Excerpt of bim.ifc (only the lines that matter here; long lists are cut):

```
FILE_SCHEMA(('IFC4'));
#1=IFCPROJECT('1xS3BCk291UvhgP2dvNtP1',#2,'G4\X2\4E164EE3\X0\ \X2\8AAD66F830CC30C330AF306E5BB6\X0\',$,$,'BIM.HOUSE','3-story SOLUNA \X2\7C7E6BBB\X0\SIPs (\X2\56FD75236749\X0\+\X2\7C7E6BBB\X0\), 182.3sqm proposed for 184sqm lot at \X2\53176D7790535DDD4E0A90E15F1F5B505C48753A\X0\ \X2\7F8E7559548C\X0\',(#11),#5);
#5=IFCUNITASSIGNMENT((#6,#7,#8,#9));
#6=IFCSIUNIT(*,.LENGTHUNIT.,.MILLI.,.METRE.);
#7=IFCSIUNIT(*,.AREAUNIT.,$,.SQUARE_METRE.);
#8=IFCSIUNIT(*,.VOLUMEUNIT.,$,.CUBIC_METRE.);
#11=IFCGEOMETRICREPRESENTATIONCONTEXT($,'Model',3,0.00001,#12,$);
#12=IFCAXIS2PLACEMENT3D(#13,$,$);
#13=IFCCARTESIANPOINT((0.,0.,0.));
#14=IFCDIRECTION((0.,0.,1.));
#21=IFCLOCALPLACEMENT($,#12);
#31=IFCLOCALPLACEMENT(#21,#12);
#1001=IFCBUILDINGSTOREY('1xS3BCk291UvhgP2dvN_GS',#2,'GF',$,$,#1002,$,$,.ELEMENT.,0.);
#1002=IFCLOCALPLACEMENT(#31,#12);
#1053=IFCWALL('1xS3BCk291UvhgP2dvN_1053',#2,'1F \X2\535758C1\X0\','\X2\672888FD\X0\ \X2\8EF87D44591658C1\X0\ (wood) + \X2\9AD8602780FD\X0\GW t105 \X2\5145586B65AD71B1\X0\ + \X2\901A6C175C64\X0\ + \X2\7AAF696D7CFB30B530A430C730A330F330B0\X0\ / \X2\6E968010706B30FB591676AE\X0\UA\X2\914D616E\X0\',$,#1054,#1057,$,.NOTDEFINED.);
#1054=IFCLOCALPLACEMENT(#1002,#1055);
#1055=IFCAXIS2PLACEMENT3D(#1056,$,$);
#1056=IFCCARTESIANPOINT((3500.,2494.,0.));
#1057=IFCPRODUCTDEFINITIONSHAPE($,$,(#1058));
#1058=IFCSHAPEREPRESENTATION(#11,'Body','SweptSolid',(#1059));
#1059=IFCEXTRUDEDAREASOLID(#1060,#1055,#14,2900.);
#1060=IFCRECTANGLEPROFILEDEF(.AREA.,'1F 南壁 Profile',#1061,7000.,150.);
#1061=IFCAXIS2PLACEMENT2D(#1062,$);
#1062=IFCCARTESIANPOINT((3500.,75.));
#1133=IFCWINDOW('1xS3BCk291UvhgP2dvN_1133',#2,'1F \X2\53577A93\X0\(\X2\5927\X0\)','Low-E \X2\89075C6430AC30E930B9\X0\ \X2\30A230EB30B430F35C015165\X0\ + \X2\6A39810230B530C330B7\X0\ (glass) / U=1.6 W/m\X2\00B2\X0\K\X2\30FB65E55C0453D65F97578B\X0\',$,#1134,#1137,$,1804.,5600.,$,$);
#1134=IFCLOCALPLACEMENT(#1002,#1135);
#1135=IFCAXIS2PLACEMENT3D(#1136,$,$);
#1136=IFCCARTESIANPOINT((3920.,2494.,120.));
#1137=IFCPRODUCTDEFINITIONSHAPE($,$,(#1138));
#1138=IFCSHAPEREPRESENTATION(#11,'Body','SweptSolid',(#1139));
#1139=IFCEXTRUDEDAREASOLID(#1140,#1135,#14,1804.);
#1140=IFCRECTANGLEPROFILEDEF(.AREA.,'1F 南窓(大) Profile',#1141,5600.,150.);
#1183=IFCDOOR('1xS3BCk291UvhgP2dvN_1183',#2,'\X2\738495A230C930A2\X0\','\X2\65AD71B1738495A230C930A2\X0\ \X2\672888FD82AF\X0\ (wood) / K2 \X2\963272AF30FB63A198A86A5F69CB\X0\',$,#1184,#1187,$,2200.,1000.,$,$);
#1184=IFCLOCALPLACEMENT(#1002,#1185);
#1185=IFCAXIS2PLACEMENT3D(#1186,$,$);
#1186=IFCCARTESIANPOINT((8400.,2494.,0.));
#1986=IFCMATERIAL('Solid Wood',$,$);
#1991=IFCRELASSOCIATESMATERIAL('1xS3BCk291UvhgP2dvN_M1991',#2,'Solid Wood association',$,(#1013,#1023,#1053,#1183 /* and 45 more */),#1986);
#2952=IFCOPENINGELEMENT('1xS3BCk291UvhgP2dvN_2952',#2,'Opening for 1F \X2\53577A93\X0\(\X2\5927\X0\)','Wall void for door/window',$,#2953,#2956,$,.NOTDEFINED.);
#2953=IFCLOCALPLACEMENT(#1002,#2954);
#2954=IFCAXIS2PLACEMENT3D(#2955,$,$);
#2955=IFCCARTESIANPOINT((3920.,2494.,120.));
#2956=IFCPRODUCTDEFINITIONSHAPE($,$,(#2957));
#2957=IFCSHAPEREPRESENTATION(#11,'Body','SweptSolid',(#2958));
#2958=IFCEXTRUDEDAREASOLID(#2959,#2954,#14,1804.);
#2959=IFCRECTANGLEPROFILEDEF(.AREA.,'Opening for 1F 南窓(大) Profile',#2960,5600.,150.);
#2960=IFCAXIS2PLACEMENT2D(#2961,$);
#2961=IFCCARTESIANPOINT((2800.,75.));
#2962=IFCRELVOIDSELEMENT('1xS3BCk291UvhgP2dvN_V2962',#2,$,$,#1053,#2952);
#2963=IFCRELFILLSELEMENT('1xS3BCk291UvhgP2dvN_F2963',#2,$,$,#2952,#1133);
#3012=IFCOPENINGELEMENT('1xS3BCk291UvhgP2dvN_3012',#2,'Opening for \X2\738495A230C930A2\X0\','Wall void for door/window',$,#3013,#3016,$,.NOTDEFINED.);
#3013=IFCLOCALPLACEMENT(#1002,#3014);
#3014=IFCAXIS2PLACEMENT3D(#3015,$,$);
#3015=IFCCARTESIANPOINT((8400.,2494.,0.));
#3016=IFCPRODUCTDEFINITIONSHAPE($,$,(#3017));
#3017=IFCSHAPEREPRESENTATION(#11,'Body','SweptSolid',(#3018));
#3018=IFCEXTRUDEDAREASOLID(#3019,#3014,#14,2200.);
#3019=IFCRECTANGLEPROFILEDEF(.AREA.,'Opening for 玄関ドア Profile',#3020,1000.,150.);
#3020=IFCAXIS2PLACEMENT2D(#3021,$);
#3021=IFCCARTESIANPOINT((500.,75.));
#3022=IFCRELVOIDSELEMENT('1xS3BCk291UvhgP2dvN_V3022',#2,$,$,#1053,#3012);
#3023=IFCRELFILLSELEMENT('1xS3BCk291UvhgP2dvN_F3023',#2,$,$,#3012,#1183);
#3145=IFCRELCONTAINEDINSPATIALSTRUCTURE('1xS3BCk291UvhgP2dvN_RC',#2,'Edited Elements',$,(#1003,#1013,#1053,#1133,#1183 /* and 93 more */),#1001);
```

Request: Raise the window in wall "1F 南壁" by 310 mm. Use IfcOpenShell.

```python
import numpy as np
import ifcopenshell
import ifcopenshell.api.geometry
import ifcopenshell.util.placement
import ifcopenshell.util.unit

model = ifcopenshell.open("bim.ifc")
unit_scale = ifcopenshell.util.unit.calculate_unit_scale(model)

window = model.by_id(1133)
opening = window.FillsVoids[0].RelatingOpeningElement
dz = 0.31 / unit_scale

shift = np.array([0.0, 0.0, dz])
# The window is not placed relative to its opening, so move both.
for product in (opening, window):
    matrix = ifcopenshell.util.placement.get_local_placement(product.ObjectPlacement)
    matrix[:3, 3] += shift
    ifcopenshell.api.geometry.edit_object_placement(model, product=product, matrix=matrix, is_si=False)

print(f"moved by {dz * unit_scale:+.3f} m")

model.write("bim_v2.ifc")
```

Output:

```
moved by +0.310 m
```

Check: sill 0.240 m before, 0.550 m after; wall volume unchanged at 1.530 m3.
